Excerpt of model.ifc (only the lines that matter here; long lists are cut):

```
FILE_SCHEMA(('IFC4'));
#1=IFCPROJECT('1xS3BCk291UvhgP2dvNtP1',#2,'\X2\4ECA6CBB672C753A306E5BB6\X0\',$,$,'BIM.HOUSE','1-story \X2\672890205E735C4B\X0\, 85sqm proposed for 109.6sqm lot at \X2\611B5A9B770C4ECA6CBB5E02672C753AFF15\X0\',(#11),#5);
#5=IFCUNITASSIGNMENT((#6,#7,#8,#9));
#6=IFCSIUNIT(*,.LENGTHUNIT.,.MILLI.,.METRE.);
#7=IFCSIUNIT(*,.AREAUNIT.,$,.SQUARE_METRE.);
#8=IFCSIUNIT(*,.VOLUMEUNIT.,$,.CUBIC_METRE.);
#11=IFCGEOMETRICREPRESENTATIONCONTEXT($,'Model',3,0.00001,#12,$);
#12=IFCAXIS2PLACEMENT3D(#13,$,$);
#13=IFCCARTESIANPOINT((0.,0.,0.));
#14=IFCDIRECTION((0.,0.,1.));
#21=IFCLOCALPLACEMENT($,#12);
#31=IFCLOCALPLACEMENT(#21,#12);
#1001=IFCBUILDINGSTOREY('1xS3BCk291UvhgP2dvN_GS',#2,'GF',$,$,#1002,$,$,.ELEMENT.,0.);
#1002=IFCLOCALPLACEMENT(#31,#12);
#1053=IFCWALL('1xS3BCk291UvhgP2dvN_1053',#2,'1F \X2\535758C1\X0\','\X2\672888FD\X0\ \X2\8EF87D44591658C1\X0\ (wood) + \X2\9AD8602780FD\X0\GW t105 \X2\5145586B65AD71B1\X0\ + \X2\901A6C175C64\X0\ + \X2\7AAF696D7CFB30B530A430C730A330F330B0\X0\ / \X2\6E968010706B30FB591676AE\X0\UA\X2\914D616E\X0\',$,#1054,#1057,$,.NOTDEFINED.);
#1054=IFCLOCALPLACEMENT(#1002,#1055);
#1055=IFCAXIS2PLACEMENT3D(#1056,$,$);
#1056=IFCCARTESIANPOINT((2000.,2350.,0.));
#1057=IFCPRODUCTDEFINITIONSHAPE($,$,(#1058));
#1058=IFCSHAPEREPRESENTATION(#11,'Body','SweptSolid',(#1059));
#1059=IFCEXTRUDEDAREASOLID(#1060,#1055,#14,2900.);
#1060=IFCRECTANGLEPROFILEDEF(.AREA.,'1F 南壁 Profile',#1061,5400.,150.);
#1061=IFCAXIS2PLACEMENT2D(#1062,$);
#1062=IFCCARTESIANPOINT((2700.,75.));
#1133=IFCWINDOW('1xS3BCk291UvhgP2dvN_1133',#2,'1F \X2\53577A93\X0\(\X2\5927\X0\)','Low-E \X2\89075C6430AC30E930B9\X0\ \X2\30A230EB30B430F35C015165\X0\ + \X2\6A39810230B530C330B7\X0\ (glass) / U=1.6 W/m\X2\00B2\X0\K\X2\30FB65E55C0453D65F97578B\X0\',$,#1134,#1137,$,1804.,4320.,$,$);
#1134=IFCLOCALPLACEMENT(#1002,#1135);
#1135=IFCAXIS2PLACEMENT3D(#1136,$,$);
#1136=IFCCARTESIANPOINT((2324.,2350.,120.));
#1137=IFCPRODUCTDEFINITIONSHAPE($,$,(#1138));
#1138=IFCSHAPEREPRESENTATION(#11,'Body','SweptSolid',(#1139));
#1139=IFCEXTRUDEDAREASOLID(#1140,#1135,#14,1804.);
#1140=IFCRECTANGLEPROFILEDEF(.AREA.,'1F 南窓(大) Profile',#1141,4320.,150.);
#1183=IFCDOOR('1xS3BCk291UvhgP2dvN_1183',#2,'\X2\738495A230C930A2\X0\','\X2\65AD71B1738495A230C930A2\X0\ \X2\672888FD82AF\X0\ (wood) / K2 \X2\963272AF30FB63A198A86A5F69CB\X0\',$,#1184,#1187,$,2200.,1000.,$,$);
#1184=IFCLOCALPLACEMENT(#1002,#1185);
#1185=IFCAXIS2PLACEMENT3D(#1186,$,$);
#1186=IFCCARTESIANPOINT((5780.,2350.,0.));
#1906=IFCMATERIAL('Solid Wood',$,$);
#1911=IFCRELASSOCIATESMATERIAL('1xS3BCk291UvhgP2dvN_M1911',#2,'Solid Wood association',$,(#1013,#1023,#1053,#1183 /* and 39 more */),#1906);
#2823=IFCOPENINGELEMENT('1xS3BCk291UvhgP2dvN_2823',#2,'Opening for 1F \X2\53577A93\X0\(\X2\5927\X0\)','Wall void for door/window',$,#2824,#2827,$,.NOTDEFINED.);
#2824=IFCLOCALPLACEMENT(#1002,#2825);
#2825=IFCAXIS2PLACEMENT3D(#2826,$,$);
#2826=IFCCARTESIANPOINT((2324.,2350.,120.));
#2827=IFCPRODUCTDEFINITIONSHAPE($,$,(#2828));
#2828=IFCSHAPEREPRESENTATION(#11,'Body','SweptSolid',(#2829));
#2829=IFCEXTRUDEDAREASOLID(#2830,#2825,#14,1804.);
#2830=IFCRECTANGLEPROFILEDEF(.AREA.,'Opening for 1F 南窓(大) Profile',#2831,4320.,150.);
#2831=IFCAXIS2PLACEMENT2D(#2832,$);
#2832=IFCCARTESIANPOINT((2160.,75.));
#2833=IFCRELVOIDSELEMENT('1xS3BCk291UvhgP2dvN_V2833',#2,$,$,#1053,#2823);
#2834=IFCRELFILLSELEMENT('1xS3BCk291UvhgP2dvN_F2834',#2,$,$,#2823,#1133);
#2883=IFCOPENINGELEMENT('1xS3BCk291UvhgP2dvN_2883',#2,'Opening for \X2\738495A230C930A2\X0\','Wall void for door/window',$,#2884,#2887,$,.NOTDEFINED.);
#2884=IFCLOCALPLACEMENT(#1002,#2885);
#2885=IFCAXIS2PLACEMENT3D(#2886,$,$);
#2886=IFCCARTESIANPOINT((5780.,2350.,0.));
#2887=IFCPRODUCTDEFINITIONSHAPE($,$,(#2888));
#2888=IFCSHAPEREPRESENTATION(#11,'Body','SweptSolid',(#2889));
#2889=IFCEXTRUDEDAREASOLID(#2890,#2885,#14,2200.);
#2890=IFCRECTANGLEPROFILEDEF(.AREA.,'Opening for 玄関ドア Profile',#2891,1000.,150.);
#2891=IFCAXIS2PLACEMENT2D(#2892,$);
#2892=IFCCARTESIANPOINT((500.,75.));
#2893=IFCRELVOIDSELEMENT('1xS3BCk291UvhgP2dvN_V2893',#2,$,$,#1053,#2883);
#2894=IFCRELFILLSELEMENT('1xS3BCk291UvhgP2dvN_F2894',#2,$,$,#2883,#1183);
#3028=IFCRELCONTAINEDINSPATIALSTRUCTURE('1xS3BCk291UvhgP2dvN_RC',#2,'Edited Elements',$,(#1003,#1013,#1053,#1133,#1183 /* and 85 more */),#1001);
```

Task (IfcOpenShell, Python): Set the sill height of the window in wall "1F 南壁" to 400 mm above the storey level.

```python
import numpy as np
import ifcopenshell
import ifcopenshell.api.geometry
import ifcopenshell.geom
import ifcopenshell.util.element
import ifcopenshell.util.placement
import ifcopenshell.util.shape
import ifcopenshell.util.unit

model = ifcopenshell.open("model.ifc")
unit_scale = ifcopenshell.util.unit.calculate_unit_scale(model)

window = model.by_guid("1xS3BCk291UvhgP2dvN_1133")
opening = window.FillsVoids[0].RelatingOpeningElement
storey = ifcopenshell.util.element.get_container(window, ifc_class="IfcBuildingStorey")
level = ifcopenshell.util.placement.get_local_placement(storey.ObjectPlacement)[2, 3]

# The opening's origin need not be at the sill, so measure its lowest point.
shape = ifcopenshell.geom.create_shape(ifcopenshell.geom.settings(), opening)
bottom = ifcopenshell.util.shape.get_shape_bottom_elevation(shape, shape.geometry) / unit_scale
dz = level + 0.4 / unit_scale - bottom

shift = np.array([0.0, 0.0, dz])
# The window is not placed relative to its opening, so move both.
for product in (opening, window):
    matrix = ifcopenshell.util.placement.get_local_placement(product.ObjectPlacement)
    matrix[:3, 3] += shift
    ifcopenshell.api.geometry.edit_object_placement(model, product=product, matrix=matrix, is_si=False)

print(f"moved by {dz * unit_scale:+.3f} m")

model.write("model_edited.ifc")
```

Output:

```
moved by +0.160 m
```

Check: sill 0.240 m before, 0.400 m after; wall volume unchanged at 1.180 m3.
